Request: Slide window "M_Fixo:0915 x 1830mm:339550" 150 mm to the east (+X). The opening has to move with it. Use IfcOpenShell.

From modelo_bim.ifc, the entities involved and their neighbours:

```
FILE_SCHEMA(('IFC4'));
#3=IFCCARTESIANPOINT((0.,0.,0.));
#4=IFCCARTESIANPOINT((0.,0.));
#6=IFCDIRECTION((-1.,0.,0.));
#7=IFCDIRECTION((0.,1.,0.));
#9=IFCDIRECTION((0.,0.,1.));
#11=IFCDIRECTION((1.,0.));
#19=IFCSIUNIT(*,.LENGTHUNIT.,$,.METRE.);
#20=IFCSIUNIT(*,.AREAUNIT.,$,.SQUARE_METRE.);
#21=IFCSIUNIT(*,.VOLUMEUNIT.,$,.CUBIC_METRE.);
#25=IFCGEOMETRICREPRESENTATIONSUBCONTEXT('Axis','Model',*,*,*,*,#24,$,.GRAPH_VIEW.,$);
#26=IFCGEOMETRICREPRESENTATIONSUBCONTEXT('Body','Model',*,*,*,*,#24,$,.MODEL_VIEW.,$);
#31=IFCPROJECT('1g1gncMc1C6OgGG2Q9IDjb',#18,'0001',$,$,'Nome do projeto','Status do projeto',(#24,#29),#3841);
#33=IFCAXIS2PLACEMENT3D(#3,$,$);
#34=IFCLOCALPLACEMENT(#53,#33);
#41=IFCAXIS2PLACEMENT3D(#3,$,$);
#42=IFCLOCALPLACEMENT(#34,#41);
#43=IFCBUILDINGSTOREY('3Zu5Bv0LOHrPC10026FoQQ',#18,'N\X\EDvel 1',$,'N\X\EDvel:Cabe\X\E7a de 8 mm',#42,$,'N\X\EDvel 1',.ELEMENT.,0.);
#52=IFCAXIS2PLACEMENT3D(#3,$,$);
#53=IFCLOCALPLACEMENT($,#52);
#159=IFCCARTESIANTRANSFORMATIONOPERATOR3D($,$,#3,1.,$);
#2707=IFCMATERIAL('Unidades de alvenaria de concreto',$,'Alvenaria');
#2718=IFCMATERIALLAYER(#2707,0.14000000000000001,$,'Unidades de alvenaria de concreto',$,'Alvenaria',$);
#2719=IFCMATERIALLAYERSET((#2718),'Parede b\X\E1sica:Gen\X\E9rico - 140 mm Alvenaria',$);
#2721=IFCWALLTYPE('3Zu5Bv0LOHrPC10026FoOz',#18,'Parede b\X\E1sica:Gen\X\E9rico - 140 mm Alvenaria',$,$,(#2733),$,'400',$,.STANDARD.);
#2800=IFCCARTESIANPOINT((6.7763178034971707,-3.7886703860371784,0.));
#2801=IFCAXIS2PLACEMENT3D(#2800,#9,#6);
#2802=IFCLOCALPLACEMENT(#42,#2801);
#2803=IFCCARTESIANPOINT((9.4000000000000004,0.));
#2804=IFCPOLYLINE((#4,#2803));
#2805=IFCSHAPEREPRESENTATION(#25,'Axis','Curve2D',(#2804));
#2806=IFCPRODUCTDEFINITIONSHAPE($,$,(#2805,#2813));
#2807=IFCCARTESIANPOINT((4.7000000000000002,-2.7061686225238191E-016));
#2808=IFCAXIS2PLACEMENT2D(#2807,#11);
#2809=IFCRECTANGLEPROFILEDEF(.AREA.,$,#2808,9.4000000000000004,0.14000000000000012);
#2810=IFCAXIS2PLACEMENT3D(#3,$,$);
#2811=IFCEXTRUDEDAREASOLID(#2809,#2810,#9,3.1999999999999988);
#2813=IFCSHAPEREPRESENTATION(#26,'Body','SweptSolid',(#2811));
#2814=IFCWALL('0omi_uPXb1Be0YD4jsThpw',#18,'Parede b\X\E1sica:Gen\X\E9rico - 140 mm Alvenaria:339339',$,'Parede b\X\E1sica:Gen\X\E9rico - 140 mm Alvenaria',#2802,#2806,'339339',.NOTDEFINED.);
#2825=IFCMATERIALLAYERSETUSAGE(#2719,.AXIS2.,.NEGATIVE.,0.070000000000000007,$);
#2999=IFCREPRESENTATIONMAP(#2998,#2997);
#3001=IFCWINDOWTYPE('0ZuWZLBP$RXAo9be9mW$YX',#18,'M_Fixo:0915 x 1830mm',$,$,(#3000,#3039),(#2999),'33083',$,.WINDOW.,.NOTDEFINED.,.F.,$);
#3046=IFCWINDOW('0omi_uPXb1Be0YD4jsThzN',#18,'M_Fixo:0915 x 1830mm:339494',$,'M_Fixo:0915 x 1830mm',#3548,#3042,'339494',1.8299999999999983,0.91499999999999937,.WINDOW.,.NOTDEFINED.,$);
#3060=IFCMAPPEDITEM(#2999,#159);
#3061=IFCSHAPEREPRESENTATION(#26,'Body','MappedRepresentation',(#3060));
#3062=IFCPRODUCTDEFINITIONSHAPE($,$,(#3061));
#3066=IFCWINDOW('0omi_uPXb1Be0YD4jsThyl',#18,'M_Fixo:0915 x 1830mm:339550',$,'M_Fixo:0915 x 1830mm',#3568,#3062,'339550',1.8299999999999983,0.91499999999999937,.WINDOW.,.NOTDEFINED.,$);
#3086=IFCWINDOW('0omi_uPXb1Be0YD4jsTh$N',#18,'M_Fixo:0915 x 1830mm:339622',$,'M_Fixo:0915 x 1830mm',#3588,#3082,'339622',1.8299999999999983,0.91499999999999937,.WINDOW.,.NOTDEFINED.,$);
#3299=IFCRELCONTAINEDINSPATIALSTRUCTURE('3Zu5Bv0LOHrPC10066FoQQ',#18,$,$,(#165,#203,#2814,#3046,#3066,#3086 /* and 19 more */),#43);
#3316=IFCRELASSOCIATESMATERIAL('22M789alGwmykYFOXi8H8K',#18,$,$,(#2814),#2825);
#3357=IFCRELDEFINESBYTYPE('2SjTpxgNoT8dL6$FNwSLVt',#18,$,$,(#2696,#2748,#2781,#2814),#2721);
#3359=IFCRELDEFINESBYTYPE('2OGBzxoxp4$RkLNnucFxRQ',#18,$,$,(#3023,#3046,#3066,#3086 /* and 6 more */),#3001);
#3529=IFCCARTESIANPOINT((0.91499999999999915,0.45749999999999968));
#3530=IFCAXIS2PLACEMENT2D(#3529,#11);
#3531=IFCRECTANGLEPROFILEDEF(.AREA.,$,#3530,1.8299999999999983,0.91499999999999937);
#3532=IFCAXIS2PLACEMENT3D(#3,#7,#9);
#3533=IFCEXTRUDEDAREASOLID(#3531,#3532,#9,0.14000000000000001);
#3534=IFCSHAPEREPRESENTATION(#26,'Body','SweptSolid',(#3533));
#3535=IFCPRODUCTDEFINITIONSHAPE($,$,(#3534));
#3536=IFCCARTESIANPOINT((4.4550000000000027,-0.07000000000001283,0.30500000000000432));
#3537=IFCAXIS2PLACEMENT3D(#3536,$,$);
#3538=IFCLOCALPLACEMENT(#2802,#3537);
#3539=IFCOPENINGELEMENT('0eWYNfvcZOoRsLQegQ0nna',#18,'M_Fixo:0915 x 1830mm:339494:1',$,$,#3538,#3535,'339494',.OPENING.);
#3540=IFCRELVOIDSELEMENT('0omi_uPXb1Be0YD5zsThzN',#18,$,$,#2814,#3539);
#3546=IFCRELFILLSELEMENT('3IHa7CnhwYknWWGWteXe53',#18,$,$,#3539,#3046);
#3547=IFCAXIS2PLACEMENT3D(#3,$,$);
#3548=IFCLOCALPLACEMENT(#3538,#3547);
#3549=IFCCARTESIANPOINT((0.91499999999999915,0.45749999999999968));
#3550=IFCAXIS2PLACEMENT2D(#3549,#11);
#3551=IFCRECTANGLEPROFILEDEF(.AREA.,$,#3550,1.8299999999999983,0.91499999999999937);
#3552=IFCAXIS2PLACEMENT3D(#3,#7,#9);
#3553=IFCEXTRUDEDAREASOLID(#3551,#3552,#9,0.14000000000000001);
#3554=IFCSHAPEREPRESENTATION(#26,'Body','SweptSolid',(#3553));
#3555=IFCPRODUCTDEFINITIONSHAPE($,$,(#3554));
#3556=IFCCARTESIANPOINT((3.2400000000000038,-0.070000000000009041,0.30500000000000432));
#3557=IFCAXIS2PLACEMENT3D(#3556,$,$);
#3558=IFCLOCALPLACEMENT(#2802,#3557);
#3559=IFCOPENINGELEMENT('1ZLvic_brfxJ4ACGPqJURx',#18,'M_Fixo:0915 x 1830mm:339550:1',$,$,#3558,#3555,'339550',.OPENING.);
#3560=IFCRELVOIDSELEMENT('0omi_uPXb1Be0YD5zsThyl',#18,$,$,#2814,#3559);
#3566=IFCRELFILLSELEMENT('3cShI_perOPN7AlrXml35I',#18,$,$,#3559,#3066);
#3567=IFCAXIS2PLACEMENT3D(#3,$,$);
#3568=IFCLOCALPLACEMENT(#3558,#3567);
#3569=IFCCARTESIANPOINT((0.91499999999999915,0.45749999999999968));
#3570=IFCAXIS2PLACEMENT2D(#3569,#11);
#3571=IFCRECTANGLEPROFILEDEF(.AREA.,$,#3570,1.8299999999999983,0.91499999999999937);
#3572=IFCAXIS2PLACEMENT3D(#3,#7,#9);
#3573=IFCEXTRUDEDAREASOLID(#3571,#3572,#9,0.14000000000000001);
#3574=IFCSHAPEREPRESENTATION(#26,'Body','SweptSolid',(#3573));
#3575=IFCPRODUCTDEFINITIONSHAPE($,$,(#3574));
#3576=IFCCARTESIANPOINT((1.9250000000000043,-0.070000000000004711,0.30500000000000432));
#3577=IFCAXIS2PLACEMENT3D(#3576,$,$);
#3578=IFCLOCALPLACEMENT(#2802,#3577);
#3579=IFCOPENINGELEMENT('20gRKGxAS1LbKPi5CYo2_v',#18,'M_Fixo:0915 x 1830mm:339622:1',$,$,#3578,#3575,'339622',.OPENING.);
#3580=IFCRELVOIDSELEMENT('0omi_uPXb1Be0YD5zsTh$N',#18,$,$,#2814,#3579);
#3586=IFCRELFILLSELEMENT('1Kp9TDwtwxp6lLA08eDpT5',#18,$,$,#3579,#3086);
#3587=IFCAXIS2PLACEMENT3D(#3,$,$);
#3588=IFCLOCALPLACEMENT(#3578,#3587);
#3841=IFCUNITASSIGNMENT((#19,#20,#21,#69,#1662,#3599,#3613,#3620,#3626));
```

```python
import ifcopenshell
import ifcopenshell.api.geometry
import ifcopenshell.util.placement

model = ifcopenshell.open("modelo_bim.ifc")

window = model.by_guid("0omi_uPXb1Be0YD4jsThyl")
opening = window.FillsVoids[0].RelatingOpeningElement
wall = opening.VoidsElements[0].RelatingBuildingElement

wall_matrix = ifcopenshell.util.placement.get_local_placement(wall.ObjectPlacement)
shift = wall_matrix[:3, 0] * -0.15
before = ifcopenshell.util.placement.get_local_placement(window.ObjectPlacement)[:3, 3].copy()

# The window is placed relative to its opening, so it follows when the opening moves.
matrix = ifcopenshell.util.placement.get_local_placement(opening.ObjectPlacement)
matrix[:3, 3] += shift
ifcopenshell.api.geometry.edit_object_placement(
    model, product=opening, matrix=matrix, is_si=False, should_transform_children=True
)

after = ifcopenshell.util.placement.get_local_placement(window.ObjectPlacement)[:3, 3]
print("window moved by", (after - before).round(3) + 0.0)

model.write("modelo_bim-out.ifc")
```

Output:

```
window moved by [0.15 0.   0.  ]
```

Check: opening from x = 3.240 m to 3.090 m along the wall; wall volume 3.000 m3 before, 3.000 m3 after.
